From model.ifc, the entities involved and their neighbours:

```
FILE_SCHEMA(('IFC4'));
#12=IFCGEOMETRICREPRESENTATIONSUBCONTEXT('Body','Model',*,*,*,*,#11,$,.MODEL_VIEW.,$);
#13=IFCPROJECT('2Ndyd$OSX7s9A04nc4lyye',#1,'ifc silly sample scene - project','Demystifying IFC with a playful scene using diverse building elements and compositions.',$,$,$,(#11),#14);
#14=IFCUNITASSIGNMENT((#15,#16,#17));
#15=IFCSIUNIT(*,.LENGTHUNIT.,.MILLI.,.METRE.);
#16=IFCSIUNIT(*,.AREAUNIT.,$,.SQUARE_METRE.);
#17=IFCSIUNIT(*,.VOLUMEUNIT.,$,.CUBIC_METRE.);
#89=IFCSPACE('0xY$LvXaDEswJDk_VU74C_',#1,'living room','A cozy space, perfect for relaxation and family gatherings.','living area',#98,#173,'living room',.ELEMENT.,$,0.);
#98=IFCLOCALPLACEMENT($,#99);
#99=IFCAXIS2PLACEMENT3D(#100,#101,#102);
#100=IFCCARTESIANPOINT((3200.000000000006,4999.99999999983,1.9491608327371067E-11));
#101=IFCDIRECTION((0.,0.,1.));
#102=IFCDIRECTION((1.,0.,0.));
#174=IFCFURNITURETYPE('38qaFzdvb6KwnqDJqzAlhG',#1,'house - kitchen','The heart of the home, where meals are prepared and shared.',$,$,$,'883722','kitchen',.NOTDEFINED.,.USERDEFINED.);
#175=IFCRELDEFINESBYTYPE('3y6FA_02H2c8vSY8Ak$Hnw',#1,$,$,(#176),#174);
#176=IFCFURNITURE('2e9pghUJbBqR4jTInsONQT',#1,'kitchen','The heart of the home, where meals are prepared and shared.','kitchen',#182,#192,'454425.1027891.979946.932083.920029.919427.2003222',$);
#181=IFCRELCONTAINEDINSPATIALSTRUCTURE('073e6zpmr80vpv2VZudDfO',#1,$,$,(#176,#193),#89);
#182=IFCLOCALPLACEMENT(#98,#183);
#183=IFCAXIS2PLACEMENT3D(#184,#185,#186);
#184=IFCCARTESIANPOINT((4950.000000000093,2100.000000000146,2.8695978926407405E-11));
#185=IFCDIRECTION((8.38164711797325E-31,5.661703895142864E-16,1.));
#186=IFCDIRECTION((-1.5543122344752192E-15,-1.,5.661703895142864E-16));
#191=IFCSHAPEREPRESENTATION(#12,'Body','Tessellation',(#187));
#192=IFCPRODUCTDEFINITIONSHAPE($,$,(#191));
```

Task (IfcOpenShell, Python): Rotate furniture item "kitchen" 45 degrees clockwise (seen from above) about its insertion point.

```python
import ifcopenshell
import ifcopenshell.api.geometry
import ifcopenshell.util.placement

model = ifcopenshell.open("model.ifc")

item = model.by_id(176)
matrix = ifcopenshell.util.placement.get_local_placement(item.ObjectPlacement)
matrix = matrix @ ifcopenshell.util.placement.rotation(-45, "Z")
ifcopenshell.api.geometry.edit_object_placement(model, product=item, matrix=matrix, is_si=False)

print(ifcopenshell.util.placement.get_local_placement(item.ObjectPlacement).round(3) + 0.0)

model.write("model-out.ifc")
```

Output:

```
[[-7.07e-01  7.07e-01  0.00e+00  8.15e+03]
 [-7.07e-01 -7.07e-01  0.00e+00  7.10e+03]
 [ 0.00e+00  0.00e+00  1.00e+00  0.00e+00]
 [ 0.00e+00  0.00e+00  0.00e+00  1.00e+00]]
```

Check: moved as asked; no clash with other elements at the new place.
